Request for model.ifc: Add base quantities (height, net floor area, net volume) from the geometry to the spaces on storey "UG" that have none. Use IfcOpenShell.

First a look at what the model holds.

```python
import ifcopenshell
import ifcopenshell.util.element
import ifcopenshell.util.unit

model = ifcopenshell.open("model.ifc")
print(model.schema)
for unit_type in ("LENGTHUNIT", "AREAUNIT", "VOLUMEUNIT"):
    print(unit_type, ifcopenshell.util.unit.calculate_unit_scale(model, unit_type))
storey = next(s for s in model.by_type("IfcBuildingStorey") if s.Name == "UG")
spaces = [e for e in ifcopenshell.util.element.get_decomposition(storey) if e.is_a("IfcSpace")]
for e in sorted(spaces, key=lambda e: e.id()):
    print(e.id(), e.is_a(), e.Name, list(ifcopenshell.util.element.get_psets(e, qtos_only=True)), sep=" | ")
```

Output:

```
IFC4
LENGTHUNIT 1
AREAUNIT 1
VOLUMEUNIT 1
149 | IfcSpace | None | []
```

```python
import ifcopenshell
import ifcopenshell.api.pset
import ifcopenshell.geom
import ifcopenshell.util.element
import ifcopenshell.util.shape
import ifcopenshell.util.unit

model = ifcopenshell.open("model.ifc")
unit_scale = ifcopenshell.util.unit.calculate_unit_scale(model)
area_scale = ifcopenshell.util.unit.calculate_unit_scale(model, "AREAUNIT")
volume_scale = ifcopenshell.util.unit.calculate_unit_scale(model, "VOLUMEUNIT")
settings = ifcopenshell.geom.settings()

storey = next(s for s in model.by_type("IfcBuildingStorey") if s.Name == "UG")
spaces = [e for e in ifcopenshell.util.element.get_decomposition(storey) if e.is_a("IfcSpace")]

for e in sorted(spaces, key=lambda e: e.id()):
    if ifcopenshell.util.element.get_psets(e, qtos_only=True, should_inherit=False):
        continue
    # Geometry comes back in metres, in the element's own axes.
    shape = ifcopenshell.geom.create_shape(settings, e)
    values = {
        "Height": ifcopenshell.util.shape.get_z(shape.geometry) / unit_scale,
        "NetFloorArea": ifcopenshell.util.shape.get_footprint_area(shape.geometry) / area_scale,
        "NetVolume": ifcopenshell.util.shape.get_volume(shape.geometry) / volume_scale,
    }
    qto = ifcopenshell.api.pset.add_qto(model, product=e, name="Qto_SpaceBaseQuantities")
    ifcopenshell.api.pset.edit_qto(model, qto=qto, properties=values)
    print(e.id(), {k: round(v, 3) for k, v in values.items()})

model.write("model_edited.ifc")
```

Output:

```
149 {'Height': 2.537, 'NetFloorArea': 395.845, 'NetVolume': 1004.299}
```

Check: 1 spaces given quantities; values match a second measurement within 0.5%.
